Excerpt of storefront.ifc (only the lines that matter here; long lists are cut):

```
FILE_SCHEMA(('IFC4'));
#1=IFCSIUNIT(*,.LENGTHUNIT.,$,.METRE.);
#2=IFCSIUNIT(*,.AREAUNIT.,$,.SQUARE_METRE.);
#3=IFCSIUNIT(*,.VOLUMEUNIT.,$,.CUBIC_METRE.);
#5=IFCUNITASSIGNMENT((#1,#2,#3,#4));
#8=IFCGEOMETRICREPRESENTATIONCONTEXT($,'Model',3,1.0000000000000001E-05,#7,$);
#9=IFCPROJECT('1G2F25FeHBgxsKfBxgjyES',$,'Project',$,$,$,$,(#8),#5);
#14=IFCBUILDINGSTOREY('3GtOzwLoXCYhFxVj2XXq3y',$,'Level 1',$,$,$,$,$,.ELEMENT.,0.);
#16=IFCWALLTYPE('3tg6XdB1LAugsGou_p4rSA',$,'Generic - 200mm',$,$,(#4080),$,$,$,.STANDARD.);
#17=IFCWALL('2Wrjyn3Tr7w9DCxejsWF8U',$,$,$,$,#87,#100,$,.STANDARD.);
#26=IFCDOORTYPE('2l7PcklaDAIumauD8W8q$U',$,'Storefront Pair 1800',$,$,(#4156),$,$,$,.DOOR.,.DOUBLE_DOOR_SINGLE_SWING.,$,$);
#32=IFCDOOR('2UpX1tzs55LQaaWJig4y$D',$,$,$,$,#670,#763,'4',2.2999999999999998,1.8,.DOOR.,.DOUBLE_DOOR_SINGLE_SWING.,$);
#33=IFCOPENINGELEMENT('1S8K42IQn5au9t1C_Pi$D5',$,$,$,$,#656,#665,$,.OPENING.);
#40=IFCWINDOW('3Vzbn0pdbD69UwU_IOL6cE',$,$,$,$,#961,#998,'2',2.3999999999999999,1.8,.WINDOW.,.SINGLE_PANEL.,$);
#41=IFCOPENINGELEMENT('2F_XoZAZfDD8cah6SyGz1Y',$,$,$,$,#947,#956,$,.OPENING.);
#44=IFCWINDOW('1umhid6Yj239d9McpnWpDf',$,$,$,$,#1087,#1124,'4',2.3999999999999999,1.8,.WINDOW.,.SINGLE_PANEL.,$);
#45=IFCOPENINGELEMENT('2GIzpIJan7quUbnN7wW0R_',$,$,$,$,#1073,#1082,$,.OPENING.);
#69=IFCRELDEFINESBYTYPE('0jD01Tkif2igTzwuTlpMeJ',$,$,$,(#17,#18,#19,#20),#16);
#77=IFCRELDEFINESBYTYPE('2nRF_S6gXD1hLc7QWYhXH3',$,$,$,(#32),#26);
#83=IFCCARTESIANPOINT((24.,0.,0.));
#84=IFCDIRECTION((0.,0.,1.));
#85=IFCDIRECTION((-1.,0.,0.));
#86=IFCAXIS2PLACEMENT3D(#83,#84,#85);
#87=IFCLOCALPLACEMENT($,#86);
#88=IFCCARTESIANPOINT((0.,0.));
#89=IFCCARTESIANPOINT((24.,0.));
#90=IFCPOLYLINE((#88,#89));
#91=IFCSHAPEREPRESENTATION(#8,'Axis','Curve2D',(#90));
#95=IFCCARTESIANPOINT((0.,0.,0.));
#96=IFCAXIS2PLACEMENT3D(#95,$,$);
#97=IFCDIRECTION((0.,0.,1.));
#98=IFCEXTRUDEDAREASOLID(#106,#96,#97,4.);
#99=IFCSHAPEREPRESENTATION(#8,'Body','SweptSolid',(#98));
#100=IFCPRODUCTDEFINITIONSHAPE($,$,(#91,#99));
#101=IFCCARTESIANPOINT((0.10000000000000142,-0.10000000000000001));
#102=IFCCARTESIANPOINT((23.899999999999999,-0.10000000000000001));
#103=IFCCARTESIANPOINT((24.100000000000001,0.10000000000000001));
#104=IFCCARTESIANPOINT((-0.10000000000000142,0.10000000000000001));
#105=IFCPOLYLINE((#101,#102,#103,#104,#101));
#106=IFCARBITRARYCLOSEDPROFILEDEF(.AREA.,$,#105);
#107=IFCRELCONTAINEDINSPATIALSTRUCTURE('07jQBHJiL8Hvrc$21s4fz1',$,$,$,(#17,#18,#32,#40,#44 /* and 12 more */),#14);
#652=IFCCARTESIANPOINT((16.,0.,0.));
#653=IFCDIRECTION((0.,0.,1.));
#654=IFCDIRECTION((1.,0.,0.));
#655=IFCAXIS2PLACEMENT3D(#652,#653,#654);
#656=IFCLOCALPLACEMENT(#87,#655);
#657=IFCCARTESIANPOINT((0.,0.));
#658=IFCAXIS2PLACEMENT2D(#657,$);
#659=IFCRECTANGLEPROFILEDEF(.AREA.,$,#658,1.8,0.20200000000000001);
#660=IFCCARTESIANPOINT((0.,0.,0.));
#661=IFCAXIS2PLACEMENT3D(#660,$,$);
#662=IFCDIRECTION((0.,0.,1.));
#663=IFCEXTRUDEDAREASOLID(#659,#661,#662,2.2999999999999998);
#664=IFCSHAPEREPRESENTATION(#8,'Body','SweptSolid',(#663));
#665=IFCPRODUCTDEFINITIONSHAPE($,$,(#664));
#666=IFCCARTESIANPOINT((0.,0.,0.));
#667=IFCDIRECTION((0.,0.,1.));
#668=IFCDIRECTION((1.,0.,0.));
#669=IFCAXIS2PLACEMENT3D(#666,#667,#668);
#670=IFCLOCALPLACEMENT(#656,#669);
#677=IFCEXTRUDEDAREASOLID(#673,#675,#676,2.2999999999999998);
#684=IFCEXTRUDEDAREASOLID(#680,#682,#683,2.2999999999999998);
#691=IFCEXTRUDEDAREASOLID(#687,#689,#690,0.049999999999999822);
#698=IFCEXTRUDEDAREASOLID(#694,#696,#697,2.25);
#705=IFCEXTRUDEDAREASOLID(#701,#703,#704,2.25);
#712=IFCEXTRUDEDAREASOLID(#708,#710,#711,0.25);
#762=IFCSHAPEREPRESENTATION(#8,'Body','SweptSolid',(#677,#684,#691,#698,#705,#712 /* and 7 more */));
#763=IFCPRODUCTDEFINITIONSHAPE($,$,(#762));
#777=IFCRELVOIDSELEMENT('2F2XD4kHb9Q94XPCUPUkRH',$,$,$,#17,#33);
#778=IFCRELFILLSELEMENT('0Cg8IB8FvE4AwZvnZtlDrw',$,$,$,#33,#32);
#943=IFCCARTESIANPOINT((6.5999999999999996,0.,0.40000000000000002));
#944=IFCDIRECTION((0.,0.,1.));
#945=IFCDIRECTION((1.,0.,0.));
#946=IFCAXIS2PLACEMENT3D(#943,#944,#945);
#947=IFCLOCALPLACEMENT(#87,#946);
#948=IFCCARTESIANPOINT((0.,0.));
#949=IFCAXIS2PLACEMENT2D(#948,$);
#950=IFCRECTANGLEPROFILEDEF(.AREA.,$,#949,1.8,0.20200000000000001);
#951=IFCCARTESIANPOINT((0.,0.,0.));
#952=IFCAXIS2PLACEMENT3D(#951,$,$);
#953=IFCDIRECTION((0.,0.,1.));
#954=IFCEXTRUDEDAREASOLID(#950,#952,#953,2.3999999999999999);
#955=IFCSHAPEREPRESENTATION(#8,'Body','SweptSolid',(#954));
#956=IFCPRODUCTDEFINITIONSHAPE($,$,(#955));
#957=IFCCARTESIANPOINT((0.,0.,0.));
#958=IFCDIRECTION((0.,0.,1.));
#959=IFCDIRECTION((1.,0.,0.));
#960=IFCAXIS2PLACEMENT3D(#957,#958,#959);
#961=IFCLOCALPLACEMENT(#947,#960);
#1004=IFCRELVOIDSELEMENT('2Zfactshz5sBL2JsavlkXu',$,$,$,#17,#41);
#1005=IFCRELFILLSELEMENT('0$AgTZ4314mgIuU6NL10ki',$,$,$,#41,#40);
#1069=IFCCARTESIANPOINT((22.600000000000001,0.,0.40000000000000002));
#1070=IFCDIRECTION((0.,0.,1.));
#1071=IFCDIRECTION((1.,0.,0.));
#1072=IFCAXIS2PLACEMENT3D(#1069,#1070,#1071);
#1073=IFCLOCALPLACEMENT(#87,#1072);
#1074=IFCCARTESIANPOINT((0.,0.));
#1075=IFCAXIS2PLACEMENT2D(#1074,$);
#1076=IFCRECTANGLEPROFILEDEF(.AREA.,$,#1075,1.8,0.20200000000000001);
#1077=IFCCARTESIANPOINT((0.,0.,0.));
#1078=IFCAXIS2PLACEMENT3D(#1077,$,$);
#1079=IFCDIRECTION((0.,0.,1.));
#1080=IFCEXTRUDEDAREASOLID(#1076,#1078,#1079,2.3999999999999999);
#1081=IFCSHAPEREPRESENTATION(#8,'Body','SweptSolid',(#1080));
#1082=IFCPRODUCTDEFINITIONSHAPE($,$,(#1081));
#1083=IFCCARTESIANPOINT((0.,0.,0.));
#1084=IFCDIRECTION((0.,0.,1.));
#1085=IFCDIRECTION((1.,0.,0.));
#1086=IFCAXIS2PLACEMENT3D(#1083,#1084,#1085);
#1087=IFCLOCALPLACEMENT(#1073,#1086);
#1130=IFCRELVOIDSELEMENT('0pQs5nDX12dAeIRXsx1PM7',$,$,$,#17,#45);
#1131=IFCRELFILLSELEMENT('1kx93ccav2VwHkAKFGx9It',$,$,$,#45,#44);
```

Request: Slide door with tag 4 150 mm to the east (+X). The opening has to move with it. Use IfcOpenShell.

```python
import ifcopenshell
import ifcopenshell.api.geometry
import ifcopenshell.util.placement
import ifcopenshell.util.unit

model = ifcopenshell.open("storefront.ifc")
unit_scale = ifcopenshell.util.unit.calculate_unit_scale(model)

door = model.by_id(32)
opening = door.FillsVoids[0].RelatingOpeningElement
wall = opening.VoidsElements[0].RelatingBuildingElement

wall_matrix = ifcopenshell.util.placement.get_local_placement(wall.ObjectPlacement)
shift = wall_matrix[:3, 0] * -0.15 / unit_scale
before = ifcopenshell.util.placement.get_local_placement(door.ObjectPlacement)[:3, 3].copy()

# The door is placed relative to its opening, so it follows when the opening moves.
matrix = ifcopenshell.util.placement.get_local_placement(opening.ObjectPlacement)
matrix[:3, 3] += shift
ifcopenshell.api.geometry.edit_object_placement(
    model, product=opening, matrix=matrix, is_si=False, should_transform_children=True
)

after = ifcopenshell.util.placement.get_local_placement(door.ObjectPlacement)[:3, 3]
print("door moved by", (after - before).round(3) + 0.0)

model.write("storefront_v2.ifc")
```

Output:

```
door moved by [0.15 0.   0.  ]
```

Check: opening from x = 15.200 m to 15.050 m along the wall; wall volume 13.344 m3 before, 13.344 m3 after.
